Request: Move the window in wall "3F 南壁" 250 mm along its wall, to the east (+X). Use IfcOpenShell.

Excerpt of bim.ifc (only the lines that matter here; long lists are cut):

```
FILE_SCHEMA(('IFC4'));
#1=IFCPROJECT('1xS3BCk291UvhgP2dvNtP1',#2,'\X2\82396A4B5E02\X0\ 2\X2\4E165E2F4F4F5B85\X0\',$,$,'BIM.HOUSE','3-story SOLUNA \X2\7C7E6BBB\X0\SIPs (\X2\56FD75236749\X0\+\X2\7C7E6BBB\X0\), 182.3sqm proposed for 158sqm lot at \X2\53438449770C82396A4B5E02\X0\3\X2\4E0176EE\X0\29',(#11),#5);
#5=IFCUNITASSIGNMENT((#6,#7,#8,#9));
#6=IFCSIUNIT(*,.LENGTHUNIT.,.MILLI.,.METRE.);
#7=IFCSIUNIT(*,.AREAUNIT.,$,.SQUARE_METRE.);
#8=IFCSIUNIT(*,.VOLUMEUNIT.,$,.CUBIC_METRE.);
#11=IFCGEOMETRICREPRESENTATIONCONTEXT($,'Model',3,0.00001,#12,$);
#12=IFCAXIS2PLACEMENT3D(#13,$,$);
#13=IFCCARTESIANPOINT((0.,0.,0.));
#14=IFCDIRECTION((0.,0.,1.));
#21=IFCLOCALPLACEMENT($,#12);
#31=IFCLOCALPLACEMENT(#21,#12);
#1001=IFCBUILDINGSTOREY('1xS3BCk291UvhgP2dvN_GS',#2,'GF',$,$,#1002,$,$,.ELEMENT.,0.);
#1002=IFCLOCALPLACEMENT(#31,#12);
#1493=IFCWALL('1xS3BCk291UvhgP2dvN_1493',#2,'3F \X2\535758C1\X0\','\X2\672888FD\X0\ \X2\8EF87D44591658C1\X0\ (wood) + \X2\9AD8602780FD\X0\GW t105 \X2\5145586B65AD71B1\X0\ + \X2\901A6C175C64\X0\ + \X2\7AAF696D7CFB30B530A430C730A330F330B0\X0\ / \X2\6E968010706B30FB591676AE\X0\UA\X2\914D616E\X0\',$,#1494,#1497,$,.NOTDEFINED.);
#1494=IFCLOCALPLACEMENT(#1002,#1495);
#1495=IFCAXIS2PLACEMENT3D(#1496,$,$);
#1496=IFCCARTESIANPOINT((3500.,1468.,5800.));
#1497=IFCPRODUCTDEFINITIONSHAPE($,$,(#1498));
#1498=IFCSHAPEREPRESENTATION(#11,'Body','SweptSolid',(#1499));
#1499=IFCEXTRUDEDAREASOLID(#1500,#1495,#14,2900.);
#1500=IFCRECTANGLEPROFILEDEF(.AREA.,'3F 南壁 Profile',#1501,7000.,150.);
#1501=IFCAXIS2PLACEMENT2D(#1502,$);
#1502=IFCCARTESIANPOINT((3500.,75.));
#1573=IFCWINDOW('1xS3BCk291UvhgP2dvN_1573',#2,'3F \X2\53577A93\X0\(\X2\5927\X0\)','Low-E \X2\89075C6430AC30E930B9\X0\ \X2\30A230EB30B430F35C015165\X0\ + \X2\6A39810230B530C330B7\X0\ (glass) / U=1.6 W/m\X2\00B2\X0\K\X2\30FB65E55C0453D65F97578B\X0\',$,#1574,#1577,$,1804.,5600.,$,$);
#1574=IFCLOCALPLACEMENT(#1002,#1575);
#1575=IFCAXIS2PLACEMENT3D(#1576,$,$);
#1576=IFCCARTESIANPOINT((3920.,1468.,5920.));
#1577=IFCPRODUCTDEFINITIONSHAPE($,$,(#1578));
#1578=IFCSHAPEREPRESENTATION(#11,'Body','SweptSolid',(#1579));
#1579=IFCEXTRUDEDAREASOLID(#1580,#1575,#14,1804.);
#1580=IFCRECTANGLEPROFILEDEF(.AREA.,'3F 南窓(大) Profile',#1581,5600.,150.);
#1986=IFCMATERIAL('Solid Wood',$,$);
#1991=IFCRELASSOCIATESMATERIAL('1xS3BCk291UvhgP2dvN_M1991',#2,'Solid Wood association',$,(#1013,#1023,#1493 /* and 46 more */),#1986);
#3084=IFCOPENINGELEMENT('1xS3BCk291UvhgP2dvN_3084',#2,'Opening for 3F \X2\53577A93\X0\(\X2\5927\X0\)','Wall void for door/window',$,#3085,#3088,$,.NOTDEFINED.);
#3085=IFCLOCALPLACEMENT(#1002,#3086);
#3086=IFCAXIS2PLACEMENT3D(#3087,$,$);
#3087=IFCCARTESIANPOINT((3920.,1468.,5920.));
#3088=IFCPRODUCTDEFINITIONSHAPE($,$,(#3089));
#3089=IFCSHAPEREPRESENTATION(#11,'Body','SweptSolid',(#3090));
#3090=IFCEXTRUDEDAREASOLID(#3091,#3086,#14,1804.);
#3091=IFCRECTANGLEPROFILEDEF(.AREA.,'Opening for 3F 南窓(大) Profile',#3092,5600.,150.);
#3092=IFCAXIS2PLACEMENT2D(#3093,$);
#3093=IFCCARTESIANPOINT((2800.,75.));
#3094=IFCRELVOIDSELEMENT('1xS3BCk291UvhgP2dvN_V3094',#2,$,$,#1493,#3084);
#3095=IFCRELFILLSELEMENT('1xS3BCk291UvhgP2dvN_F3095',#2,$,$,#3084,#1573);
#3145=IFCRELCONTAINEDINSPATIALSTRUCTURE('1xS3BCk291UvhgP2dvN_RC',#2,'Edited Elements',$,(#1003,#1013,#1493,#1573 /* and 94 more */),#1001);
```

```python
import ifcopenshell
import ifcopenshell.api.geometry
import ifcopenshell.util.placement

model = ifcopenshell.open("bim.ifc")

window = model.by_id(1573)
opening = window.FillsVoids[0].RelatingOpeningElement
wall = opening.VoidsElements[0].RelatingBuildingElement

wall_matrix = ifcopenshell.util.placement.get_local_placement(wall.ObjectPlacement)
shift = wall_matrix[:3, 0] * 250.0
before = ifcopenshell.util.placement.get_local_placement(window.ObjectPlacement)[:3, 3].copy()

# The window is not placed relative to its opening, so move both.
for product in (opening, window):
    matrix = ifcopenshell.util.placement.get_local_placement(product.ObjectPlacement)
    matrix[:3, 3] += shift
    ifcopenshell.api.geometry.edit_object_placement(model, product=product, matrix=matrix, is_si=False)

after = ifcopenshell.util.placement.get_local_placement(window.ObjectPlacement)[:3, 3]
print("window moved by", (after - before).round(3) + 0.0)

model.write("bim_v2.ifc")
```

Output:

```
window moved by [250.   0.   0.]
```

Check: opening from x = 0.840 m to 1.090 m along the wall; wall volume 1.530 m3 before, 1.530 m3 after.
